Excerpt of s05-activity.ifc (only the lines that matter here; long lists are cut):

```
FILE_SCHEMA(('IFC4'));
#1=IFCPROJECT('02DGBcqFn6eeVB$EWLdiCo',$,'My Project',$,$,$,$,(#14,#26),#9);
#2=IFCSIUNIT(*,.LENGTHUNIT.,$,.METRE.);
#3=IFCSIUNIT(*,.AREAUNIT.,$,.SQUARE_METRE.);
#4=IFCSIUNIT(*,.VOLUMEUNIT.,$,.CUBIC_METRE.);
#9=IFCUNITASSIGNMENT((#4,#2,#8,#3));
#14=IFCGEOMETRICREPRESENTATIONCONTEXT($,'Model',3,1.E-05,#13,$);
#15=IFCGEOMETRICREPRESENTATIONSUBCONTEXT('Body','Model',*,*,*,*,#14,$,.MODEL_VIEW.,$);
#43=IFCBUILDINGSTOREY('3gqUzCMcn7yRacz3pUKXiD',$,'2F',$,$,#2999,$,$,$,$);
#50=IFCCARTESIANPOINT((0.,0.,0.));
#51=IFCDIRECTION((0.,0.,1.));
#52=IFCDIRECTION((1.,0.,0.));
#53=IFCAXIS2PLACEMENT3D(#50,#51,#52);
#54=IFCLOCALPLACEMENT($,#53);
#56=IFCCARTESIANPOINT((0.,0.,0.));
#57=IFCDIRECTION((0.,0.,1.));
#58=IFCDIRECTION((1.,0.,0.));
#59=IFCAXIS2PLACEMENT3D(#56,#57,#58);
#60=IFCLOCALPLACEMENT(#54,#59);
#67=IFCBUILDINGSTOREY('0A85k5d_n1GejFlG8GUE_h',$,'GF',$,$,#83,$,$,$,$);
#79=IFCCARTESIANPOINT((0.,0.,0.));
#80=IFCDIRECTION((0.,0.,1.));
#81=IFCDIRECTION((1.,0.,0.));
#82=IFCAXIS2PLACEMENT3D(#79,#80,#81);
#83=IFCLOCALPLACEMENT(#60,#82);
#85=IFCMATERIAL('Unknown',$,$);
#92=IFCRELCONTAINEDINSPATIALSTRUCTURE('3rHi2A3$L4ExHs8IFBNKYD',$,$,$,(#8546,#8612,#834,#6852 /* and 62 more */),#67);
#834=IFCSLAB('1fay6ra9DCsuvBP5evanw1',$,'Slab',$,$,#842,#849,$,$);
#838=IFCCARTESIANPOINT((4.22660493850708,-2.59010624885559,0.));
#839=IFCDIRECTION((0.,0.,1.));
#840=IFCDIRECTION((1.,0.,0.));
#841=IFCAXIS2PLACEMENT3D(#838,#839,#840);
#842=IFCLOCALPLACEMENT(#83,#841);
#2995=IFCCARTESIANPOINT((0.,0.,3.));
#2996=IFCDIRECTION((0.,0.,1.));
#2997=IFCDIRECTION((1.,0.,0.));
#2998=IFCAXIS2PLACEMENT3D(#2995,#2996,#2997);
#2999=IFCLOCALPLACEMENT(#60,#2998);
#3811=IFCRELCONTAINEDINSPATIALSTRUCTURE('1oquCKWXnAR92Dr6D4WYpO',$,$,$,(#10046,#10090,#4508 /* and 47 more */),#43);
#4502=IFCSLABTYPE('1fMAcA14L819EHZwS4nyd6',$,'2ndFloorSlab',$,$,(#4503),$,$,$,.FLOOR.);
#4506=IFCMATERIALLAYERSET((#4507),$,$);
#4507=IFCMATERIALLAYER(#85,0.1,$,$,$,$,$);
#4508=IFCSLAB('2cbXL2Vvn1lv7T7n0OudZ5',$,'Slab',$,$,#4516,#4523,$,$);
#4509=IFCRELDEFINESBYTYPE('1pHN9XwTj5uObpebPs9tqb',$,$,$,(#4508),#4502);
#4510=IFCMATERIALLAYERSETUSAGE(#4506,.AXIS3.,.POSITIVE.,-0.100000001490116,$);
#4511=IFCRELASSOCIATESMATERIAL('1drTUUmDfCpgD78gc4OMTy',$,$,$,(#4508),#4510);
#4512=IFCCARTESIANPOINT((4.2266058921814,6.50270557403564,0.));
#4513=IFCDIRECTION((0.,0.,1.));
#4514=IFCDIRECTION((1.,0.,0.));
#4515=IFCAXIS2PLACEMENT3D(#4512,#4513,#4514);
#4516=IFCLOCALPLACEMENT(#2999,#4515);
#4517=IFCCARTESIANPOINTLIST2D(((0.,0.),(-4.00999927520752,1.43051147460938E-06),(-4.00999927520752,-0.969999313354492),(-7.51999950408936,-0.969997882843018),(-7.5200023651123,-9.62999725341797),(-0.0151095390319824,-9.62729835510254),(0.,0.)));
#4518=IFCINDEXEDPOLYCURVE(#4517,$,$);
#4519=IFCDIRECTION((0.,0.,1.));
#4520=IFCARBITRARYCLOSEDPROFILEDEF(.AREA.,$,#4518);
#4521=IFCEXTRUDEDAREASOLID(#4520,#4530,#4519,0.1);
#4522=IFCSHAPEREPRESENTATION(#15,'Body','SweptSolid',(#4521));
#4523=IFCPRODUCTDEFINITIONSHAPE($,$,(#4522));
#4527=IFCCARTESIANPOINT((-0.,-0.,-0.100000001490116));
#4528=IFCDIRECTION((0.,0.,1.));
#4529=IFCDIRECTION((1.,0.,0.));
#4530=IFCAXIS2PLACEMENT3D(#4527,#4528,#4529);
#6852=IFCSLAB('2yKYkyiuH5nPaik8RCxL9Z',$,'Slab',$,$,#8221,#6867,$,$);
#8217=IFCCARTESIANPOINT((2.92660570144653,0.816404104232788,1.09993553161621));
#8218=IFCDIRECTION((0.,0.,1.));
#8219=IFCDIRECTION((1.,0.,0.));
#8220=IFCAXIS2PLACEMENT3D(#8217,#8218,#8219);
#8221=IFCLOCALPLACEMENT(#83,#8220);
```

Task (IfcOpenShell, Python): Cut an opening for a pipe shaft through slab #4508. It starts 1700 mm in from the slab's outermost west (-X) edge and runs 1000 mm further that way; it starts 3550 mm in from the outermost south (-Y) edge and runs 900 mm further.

```python
import numpy as np
import ifcopenshell
import ifcopenshell.api.feature
import ifcopenshell.api.geometry
import ifcopenshell.api.root
import ifcopenshell.geom
import ifcopenshell.util.placement
import ifcopenshell.util.representation
import ifcopenshell.util.shape
import ifcopenshell.util.unit

model = ifcopenshell.open("s05-activity.ifc")
unit_scale = ifcopenshell.util.unit.calculate_unit_scale(model)
settings = ifcopenshell.geom.settings()


def volume(element):
    """Net volume in cubic metres, openings subtracted."""
    shape = ifcopenshell.geom.create_shape(settings, element)
    return ifcopenshell.util.shape.get_volume(shape.geometry)


slab = model.by_id(4508)
before = volume(slab)

# Extent in the slab's own axes, in metres. The edges named are its -X and -Y sides.
slab_shape = ifcopenshell.geom.create_shape(settings, slab)
vertices = ifcopenshell.util.shape.get_vertices(slab_shape.geometry)
x_min, y_min, bottom = vertices.min(axis=0)
top = vertices[:, 2].max()

opening = ifcopenshell.api.root.create_entity(model, ifc_class="IfcOpeningElement", name="Pipe shaft opening", predefined_type="OPENING")
context = ifcopenshell.util.representation.get_context(model, "Model", "Body", "MODEL_VIEW")
width, depth = 1, 0.9
outline = [(0.0, 0.0), (width, 0.0), (width, depth), (0.0, depth), (0.0, 0.0)]
# Overshoot both faces by 50 mm so the cut is clean.
shape = ifcopenshell.api.geometry.add_slab_representation(
    model, context=context, depth=top - bottom + 0.1, polyline=outline
)
ifcopenshell.api.geometry.assign_representation(model, product=opening, representation=shape)

matrix = ifcopenshell.util.placement.get_local_placement(slab.ObjectPlacement)
matrix[:, 3] = matrix @ np.append(np.array([x_min + 1.7, y_min + 3.55, bottom - 0.05]) / unit_scale, 1.0)
ifcopenshell.api.geometry.edit_object_placement(model, product=opening, matrix=matrix, is_si=False)
ifcopenshell.api.feature.add_feature(model, feature=opening, element=slab)

after = volume(slab)

print(f"slab volume {before:.3f} -> {after:.3f} m3")

model.write("s05-activity_edited.ifc")
```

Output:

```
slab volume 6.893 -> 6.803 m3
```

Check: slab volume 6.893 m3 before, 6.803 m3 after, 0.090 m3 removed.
